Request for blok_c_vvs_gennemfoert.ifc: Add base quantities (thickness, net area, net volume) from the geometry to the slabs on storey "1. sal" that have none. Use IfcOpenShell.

First a look at what the model holds.

```python
import ifcopenshell
import ifcopenshell.util.element
import ifcopenshell.util.unit

model = ifcopenshell.open("blok_c_vvs_gennemfoert.ifc")
print(model.schema)
for unit_type in ("LENGTHUNIT", "AREAUNIT", "VOLUMEUNIT"):
    print(unit_type, ifcopenshell.util.unit.calculate_unit_scale(model, unit_type))
storey = next(s for s in model.by_type("IfcBuildingStorey") if s.Name == "1. sal")
slabs = [e for e in ifcopenshell.util.element.get_decomposition(storey) if e.is_a("IfcSlab")]
for e in sorted(slabs, key=lambda e: e.id()):
    print(e.id(), e.is_a(), e.Name, list(ifcopenshell.util.element.get_psets(e, qtos_only=True)), sep=" | ")
```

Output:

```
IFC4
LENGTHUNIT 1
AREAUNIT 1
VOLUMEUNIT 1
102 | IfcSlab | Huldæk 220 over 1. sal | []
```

```python
import ifcopenshell
import ifcopenshell.api.pset
import ifcopenshell.geom
import ifcopenshell.util.element
import ifcopenshell.util.shape
import ifcopenshell.util.unit

model = ifcopenshell.open("blok_c_vvs_gennemfoert.ifc")
unit_scale = ifcopenshell.util.unit.calculate_unit_scale(model)
area_scale = ifcopenshell.util.unit.calculate_unit_scale(model, "AREAUNIT")
volume_scale = ifcopenshell.util.unit.calculate_unit_scale(model, "VOLUMEUNIT")
settings = ifcopenshell.geom.settings()

storey = next(s for s in model.by_type("IfcBuildingStorey") if s.Name == "1. sal")
slabs = [e for e in ifcopenshell.util.element.get_decomposition(storey) if e.is_a("IfcSlab")]

for e in sorted(slabs, key=lambda e: e.id()):
    if ifcopenshell.util.element.get_psets(e, qtos_only=True, should_inherit=False):
        continue
    # Geometry comes back in metres, in the element's own axes.
    shape = ifcopenshell.geom.create_shape(settings, e)
    values = {
        "Width": ifcopenshell.util.shape.get_z(shape.geometry) / unit_scale,
        "NetArea": ifcopenshell.util.shape.get_footprint_area(shape.geometry) / area_scale,
        "NetVolume": ifcopenshell.util.shape.get_volume(shape.geometry) / volume_scale,
    }
    qto = ifcopenshell.api.pset.add_qto(model, product=e, name="Qto_SlabBaseQuantities")
    ifcopenshell.api.pset.edit_qto(model, qto=qto, properties=values)
    print(e.id(), {k: round(v, 3) for k, v in values.items()})

model.write("blok_c_vvs_gennemfoert-out.ifc")
```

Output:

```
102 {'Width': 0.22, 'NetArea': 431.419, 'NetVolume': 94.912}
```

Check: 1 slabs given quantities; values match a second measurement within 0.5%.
